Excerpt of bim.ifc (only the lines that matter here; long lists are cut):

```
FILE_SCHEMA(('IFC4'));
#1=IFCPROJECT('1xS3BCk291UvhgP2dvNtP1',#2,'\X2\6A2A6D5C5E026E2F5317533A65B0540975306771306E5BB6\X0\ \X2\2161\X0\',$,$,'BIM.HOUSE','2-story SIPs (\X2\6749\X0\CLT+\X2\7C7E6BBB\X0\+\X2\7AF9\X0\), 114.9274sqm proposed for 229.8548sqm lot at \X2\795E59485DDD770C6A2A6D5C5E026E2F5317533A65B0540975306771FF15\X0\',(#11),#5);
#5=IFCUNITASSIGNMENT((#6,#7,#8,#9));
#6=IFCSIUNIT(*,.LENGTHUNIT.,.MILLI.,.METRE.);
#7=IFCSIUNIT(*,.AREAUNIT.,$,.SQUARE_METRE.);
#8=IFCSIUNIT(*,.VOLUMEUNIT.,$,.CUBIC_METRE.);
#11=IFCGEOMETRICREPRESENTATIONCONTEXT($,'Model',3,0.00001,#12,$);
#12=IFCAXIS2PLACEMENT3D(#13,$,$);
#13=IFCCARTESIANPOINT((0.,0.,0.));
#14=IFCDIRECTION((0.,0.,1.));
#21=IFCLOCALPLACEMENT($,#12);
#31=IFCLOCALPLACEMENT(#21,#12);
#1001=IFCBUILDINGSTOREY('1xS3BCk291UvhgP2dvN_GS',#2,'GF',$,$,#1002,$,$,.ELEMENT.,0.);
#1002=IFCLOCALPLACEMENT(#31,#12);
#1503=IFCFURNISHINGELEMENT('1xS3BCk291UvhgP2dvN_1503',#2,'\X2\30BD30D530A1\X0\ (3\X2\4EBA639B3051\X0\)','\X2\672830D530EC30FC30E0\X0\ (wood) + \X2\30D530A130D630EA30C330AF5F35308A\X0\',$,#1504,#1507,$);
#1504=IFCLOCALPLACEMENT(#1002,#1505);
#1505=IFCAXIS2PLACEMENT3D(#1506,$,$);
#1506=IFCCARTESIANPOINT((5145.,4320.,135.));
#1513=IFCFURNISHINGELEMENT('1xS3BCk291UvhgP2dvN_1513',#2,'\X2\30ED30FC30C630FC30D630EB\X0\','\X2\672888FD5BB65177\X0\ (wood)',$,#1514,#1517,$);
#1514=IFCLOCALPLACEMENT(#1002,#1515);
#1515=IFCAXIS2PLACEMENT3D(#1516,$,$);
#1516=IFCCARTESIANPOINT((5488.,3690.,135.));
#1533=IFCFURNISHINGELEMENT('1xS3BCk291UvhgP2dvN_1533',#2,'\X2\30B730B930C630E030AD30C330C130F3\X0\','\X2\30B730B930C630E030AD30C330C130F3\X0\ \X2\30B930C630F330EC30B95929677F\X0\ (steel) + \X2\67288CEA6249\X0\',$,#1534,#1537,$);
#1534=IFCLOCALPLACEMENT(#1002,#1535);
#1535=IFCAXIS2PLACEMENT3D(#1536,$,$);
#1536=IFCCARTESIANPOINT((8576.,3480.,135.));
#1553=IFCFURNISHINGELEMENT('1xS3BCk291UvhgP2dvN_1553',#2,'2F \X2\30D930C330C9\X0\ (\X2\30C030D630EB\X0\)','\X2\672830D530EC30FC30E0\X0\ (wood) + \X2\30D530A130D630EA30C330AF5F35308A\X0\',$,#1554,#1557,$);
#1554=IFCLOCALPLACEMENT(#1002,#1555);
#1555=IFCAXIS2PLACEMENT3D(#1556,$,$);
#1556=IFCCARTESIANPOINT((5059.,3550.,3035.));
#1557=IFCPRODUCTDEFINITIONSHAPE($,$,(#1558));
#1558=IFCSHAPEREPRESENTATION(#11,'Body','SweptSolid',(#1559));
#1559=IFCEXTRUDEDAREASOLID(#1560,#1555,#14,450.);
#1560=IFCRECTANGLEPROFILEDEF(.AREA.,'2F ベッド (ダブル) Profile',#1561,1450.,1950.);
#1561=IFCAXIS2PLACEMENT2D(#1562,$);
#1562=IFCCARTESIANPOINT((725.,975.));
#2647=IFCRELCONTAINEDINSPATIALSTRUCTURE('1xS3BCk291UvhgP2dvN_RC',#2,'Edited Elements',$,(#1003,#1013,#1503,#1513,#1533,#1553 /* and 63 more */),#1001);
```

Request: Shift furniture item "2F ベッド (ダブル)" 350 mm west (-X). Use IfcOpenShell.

```python
import ifcopenshell
import ifcopenshell.api.geometry
import ifcopenshell.util.placement
import ifcopenshell.util.unit

model = ifcopenshell.open("bim.ifc")
unit_scale = ifcopenshell.util.unit.calculate_unit_scale(model)

item = model.by_id(1553)
matrix = ifcopenshell.util.placement.get_local_placement(item.ObjectPlacement)
matrix[0, 3] -= 0.35 / unit_scale
ifcopenshell.api.geometry.edit_object_placement(model, product=item, matrix=matrix, is_si=False)

print(ifcopenshell.util.placement.get_local_placement(item.ObjectPlacement).round(3) + 0.0)

model.write("bim_rev.ifc")
```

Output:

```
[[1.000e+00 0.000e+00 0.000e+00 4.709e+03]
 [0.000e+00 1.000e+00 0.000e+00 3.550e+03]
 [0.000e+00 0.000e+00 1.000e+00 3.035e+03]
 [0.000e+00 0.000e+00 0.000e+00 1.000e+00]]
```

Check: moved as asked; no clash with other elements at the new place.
